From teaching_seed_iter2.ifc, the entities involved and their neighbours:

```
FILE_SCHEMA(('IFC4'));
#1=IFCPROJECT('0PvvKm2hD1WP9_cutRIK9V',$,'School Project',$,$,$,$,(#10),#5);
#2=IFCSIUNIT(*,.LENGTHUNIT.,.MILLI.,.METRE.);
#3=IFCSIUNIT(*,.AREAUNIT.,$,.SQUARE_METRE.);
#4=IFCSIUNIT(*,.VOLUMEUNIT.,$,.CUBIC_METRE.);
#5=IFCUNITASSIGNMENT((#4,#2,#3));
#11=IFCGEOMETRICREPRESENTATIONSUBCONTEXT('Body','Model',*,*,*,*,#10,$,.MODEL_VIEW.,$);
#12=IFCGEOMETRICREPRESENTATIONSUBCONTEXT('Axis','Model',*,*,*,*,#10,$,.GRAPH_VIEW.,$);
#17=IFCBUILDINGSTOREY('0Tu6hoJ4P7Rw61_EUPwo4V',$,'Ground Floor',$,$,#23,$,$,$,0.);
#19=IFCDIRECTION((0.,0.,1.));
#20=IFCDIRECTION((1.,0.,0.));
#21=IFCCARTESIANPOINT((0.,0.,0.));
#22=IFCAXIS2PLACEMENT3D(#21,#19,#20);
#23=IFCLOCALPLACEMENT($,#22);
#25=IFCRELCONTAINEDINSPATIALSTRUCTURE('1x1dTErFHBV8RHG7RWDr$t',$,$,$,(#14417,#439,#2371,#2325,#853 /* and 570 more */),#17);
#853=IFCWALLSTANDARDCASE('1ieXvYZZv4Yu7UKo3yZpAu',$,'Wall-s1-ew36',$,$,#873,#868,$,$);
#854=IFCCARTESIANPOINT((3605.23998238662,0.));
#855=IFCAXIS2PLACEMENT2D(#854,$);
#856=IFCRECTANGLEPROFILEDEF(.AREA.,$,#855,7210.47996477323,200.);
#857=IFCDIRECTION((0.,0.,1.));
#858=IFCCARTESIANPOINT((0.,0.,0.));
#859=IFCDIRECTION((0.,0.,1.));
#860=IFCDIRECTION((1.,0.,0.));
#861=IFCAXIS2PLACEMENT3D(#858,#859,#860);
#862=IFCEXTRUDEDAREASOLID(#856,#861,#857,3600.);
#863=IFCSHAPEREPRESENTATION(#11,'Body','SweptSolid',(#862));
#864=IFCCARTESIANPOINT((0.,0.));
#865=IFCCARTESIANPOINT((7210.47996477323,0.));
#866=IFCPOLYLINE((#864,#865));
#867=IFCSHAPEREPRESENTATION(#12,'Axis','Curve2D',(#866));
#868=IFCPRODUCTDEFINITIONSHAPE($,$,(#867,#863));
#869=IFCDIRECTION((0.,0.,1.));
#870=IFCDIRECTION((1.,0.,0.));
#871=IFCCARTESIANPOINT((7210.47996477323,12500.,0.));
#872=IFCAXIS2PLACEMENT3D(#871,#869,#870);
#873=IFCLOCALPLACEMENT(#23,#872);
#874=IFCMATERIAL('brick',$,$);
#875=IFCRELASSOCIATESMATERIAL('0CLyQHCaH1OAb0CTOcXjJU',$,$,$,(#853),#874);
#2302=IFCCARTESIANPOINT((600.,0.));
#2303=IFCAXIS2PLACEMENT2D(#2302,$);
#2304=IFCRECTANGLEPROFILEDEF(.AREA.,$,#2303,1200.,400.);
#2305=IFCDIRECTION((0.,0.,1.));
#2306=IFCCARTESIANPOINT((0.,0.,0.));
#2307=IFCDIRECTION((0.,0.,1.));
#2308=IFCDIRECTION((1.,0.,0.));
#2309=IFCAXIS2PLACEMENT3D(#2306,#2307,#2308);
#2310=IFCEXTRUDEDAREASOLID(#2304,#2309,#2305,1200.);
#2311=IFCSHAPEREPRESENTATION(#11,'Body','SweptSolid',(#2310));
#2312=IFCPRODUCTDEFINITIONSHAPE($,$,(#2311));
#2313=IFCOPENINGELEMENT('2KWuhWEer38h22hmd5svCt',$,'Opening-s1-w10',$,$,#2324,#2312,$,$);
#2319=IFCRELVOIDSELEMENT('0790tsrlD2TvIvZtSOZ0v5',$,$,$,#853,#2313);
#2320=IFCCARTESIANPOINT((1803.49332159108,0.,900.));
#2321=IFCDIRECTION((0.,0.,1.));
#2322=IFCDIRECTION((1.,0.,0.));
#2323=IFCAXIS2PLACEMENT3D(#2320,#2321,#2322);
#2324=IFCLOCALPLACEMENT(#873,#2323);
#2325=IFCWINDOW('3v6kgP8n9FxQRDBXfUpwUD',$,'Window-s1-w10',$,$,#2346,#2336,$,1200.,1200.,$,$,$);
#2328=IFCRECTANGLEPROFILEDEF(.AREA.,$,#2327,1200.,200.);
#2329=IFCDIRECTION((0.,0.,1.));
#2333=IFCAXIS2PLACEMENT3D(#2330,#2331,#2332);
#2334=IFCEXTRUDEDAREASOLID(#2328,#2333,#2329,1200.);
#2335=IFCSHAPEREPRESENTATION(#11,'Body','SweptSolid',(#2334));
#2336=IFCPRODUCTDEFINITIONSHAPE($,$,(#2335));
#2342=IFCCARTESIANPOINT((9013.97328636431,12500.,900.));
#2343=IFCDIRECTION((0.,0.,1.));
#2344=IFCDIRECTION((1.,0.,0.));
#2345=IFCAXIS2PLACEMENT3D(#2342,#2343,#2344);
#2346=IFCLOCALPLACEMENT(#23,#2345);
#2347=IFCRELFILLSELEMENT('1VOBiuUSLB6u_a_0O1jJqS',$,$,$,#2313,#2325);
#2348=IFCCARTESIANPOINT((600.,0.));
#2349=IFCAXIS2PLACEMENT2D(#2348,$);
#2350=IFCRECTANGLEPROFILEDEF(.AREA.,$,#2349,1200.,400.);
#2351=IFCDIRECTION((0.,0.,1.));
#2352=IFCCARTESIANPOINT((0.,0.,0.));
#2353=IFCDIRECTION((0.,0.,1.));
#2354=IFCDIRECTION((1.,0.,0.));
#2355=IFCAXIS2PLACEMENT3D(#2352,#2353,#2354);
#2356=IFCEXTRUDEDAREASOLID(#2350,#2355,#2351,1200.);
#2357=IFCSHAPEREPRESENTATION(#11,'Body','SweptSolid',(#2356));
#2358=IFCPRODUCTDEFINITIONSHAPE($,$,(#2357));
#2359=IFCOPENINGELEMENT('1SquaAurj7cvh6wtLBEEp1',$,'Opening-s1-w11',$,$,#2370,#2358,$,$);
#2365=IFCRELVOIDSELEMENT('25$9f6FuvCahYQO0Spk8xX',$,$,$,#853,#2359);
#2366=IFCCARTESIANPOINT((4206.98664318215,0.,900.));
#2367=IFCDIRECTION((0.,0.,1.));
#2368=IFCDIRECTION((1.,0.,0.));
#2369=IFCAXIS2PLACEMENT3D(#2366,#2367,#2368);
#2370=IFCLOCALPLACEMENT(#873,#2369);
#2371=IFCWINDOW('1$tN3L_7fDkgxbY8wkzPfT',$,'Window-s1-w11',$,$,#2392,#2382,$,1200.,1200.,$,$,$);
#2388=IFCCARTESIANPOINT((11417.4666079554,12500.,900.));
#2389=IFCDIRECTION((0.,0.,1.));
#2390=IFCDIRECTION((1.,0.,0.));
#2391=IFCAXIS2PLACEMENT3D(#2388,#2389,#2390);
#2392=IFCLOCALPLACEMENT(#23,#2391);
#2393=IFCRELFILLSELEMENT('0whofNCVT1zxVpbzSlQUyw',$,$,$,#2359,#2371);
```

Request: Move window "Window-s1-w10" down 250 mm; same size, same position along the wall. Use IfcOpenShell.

```python
import numpy as np
import ifcopenshell
import ifcopenshell.api.geometry
import ifcopenshell.util.placement
import ifcopenshell.util.unit

model = ifcopenshell.open("teaching_seed_iter2.ifc")
unit_scale = ifcopenshell.util.unit.calculate_unit_scale(model)

window = model.by_id(2325)
opening = window.FillsVoids[0].RelatingOpeningElement
dz = -0.25 / unit_scale

shift = np.array([0.0, 0.0, dz])
# The window is not placed relative to its opening, so move both.
for product in (opening, window):
    matrix = ifcopenshell.util.placement.get_local_placement(product.ObjectPlacement)
    matrix[:3, 3] += shift
    ifcopenshell.api.geometry.edit_object_placement(model, product=product, matrix=matrix, is_si=False)

print(f"moved by {dz * unit_scale:+.3f} m")

model.write("teaching_seed_iter2_v2.ifc")
```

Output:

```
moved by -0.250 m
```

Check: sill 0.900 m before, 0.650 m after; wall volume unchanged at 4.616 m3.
